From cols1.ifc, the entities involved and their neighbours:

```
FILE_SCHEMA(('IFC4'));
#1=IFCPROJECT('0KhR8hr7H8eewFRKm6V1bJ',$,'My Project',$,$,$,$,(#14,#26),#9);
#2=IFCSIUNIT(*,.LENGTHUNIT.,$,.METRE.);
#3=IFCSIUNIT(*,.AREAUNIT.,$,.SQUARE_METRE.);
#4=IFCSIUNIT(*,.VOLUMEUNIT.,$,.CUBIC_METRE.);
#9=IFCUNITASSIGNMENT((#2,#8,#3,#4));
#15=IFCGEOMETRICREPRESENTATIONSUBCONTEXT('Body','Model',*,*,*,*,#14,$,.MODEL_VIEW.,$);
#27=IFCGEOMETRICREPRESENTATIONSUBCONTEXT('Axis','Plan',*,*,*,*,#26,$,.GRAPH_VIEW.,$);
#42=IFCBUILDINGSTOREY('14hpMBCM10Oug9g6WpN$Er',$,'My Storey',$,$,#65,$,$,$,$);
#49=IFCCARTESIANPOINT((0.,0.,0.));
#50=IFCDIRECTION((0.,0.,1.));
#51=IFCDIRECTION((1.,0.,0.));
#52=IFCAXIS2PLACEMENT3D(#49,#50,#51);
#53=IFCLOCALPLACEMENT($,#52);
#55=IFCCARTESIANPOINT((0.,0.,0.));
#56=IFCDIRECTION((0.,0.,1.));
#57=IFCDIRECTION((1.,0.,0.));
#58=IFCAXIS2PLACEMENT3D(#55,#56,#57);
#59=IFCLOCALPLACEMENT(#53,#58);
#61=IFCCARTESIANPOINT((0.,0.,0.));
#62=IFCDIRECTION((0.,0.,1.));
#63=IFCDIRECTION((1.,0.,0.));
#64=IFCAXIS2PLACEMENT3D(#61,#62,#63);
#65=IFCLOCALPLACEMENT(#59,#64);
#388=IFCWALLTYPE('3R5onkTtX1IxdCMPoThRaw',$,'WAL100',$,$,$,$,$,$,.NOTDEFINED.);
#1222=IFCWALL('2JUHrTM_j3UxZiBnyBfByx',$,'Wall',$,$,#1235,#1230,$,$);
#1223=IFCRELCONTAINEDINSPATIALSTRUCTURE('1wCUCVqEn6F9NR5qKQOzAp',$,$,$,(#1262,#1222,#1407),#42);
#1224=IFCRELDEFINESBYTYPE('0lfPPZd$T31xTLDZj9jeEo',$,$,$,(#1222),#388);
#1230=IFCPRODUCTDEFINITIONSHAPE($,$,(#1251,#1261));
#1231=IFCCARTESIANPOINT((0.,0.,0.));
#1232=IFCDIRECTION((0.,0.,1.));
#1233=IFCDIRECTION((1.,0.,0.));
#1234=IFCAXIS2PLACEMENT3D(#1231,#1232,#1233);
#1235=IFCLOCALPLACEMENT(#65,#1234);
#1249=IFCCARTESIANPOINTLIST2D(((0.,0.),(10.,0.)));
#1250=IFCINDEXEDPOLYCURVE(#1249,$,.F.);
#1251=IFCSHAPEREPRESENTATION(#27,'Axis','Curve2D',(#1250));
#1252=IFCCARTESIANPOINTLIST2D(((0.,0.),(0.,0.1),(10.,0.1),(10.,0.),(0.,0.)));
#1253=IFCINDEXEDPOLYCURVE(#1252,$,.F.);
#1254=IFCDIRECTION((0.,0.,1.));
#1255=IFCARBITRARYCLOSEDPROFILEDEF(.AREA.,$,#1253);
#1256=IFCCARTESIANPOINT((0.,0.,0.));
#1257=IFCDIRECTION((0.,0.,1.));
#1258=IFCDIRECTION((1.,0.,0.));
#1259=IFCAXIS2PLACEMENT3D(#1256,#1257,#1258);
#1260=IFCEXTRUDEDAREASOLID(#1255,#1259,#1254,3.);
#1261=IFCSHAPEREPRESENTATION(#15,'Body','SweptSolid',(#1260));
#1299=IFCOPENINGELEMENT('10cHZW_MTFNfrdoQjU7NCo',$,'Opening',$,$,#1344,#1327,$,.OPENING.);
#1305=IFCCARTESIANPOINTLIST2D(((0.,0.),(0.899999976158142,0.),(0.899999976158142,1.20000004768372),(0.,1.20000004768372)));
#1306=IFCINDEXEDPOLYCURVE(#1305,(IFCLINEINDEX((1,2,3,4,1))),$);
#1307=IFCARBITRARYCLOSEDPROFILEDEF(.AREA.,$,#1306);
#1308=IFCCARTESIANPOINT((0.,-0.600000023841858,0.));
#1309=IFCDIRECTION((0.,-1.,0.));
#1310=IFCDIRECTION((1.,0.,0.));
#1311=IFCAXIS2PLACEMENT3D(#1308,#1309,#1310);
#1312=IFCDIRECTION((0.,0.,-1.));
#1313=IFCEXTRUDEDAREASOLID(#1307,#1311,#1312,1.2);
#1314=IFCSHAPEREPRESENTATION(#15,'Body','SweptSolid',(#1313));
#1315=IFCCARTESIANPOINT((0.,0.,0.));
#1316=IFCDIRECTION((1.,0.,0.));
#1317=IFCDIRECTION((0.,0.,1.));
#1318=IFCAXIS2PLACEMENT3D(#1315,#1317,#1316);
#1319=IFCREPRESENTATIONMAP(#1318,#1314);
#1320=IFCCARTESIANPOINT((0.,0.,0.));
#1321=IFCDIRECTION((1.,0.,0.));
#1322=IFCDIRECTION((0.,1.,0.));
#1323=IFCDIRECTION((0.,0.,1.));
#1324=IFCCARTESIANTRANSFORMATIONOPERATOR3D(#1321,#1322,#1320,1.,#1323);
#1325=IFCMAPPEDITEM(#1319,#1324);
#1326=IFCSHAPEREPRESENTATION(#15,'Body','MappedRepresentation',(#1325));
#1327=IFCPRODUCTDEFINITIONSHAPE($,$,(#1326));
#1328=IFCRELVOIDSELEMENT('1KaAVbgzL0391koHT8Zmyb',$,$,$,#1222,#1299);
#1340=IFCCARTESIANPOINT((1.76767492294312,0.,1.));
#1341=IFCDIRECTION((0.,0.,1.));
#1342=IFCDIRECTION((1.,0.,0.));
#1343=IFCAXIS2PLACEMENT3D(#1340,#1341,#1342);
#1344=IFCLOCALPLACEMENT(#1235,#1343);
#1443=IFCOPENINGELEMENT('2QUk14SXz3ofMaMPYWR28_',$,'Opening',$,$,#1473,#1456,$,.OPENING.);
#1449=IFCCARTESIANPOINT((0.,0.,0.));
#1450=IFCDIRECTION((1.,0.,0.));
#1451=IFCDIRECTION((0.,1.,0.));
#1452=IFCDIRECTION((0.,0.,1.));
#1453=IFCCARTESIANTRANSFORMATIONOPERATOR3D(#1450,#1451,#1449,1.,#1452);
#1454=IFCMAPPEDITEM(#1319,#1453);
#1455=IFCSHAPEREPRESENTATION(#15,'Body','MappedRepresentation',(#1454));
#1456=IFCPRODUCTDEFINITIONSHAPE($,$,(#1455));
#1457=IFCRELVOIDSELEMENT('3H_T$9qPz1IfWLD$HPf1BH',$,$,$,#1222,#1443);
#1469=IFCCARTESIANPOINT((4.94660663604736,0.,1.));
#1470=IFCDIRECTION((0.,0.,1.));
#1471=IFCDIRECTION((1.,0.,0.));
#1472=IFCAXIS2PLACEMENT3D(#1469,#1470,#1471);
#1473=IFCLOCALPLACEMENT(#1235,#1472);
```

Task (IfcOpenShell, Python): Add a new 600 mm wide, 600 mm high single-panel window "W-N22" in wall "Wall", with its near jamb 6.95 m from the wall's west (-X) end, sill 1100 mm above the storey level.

```python
import numpy as np
import ifcopenshell
import ifcopenshell.api.feature
import ifcopenshell.api.geometry
import ifcopenshell.api.root
import ifcopenshell.api.spatial
import ifcopenshell.geom
import ifcopenshell.util.element
import ifcopenshell.util.placement
import ifcopenshell.util.representation
import ifcopenshell.util.shape
import ifcopenshell.util.unit

model = ifcopenshell.open("cols1.ifc")
unit_scale = ifcopenshell.util.unit.calculate_unit_scale(model)
settings = ifcopenshell.geom.settings()


def volume(element):
    """Net volume in cubic metres, openings subtracted."""
    shape = ifcopenshell.geom.create_shape(settings, element)
    return ifcopenshell.util.shape.get_volume(shape.geometry)


wall = model.by_guid("2JUHrTM_j3UxZiBnyBfByx")
storey = ifcopenshell.util.element.get_container(wall, ifc_class="IfcBuildingStorey")
context = ifcopenshell.util.representation.get_context(model, "Model", "Body", "MODEL_VIEW")
before = volume(wall)

width, height, from_end, sill = 0.6, 0.6, 6.95, 1.1  # metres

# The wall runs along its own X axis, and the end named is its -X end.
wall_shape = ifcopenshell.geom.create_shape(settings, wall)
x, y, z = ifcopenshell.util.shape.get_vertices(wall_shape.geometry).T
start = x.min() + from_end
face, thickness = float(y.min()), float(y.max() - y.min())
wall_matrix = ifcopenshell.util.placement.get_local_placement(wall.ObjectPlacement)
level = ifcopenshell.util.placement.get_local_placement(storey.ObjectPlacement)[2, 3]


def in_wall(x, y):
    """Placement at x, y metres in the wall's axes, at sill height."""
    matrix = wall_matrix.copy()
    matrix[:, 3] = wall_matrix @ np.array([x / unit_scale, y / unit_scale, 0.0, 1.0])
    matrix[2, 3] = level + sill / unit_scale
    return matrix


# Opening: a box that overshoots both wall faces by 50 mm.
opening = ifcopenshell.api.root.create_entity(model, ifc_class="IfcOpeningElement", predefined_type="OPENING")
box = ifcopenshell.api.geometry.add_wall_representation(
    model, context=context, length=width, height=height, thickness=thickness + 0.1
)
ifcopenshell.api.geometry.assign_representation(model, product=opening, representation=box)
ifcopenshell.api.geometry.edit_object_placement(model, product=opening, matrix=in_wall(start, face - 0.05), is_si=False)
ifcopenshell.api.feature.add_feature(model, feature=opening, element=wall)

window = ifcopenshell.api.root.create_entity(model, ifc_class="IfcWindow", name="W-N22", predefined_type="WINDOW")
window.OverallWidth, window.OverallHeight = width / unit_scale, height / unit_scale
window.PartitioningType = "SINGLE_PANEL"
body = ifcopenshell.api.geometry.add_window_representation(
    model,
    context=context,
    overall_width=window.OverallWidth,
    overall_height=window.OverallHeight,
    partition_type="SINGLE_PANEL",
)
ifcopenshell.api.geometry.assign_representation(model, product=window, representation=body)
ifcopenshell.api.spatial.assign_container(model, products=[window], relating_structure=storey)
ifcopenshell.api.feature.add_filling(model, opening=opening, element=window)

# Centre the window in the wall's thickness.
ifcopenshell.api.geometry.edit_object_placement(model, product=window, matrix=in_wall(start, face), is_si=False)
window_shape = ifcopenshell.geom.create_shape(settings, window)
depth = ifcopenshell.util.shape.get_vertices(window_shape.geometry)[:, 1]
offset = face + thickness / 2 - (depth.min() + depth.max()) / 2
ifcopenshell.api.geometry.edit_object_placement(model, product=window, matrix=in_wall(start, offset), is_si=False)

after = volume(wall)

print(f"wall volume {before:.3f} -> {after:.3f} m3")

model.write("cols1_rev.ifc")
```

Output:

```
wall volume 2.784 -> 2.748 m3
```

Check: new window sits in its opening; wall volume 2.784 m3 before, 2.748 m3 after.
